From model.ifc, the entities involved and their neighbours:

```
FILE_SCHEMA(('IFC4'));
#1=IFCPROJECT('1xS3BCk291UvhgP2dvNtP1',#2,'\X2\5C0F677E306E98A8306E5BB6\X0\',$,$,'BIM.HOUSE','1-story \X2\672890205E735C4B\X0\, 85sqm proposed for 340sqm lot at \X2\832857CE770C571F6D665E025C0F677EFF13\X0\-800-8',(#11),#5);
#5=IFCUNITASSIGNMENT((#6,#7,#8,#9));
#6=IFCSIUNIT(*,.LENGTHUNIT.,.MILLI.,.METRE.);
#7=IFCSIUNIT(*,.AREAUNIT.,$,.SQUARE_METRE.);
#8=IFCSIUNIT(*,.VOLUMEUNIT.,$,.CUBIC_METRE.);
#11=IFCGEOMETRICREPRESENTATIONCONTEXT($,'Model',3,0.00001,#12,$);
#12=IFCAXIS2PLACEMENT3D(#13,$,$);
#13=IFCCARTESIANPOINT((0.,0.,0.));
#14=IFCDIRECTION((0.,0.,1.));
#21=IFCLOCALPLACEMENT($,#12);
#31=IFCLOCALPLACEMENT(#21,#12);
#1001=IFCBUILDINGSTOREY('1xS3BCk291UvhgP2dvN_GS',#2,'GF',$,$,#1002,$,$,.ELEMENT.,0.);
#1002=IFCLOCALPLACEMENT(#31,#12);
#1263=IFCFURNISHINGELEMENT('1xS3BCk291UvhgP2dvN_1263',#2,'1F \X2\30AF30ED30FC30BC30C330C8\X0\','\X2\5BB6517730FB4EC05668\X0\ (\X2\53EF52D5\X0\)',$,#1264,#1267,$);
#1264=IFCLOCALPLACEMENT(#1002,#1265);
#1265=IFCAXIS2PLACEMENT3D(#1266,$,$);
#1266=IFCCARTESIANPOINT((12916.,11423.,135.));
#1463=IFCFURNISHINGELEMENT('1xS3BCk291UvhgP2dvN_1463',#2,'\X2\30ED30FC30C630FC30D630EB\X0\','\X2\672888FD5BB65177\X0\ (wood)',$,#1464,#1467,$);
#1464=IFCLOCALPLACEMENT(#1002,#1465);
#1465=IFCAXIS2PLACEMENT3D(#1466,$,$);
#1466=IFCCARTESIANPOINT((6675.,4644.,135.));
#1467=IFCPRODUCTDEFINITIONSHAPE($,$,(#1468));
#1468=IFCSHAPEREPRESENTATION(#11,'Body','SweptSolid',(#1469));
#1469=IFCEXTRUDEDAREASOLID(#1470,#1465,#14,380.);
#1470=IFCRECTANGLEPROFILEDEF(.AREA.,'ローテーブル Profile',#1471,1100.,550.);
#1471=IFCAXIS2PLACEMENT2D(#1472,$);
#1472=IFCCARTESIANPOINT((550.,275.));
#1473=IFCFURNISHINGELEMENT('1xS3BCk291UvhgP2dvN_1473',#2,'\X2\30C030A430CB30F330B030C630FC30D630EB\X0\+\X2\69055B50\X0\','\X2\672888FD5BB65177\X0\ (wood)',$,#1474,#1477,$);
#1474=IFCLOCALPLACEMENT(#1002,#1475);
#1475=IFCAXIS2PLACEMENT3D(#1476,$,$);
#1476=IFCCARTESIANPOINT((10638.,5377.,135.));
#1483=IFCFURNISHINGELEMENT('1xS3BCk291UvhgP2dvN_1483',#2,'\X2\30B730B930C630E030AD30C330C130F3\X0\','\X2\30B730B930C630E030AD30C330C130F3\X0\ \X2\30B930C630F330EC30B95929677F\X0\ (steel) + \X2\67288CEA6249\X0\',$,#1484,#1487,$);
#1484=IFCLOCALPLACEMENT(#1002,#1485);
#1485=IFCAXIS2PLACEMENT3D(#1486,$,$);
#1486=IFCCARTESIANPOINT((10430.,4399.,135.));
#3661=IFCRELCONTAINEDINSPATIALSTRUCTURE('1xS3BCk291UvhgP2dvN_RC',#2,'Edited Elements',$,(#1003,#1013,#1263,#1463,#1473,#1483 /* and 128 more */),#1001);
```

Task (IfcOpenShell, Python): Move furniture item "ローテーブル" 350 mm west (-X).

```python
import ifcopenshell
import ifcopenshell.api.geometry
import ifcopenshell.util.placement

model = ifcopenshell.open("model.ifc")

item = model.by_id(1463)
matrix = ifcopenshell.util.placement.get_local_placement(item.ObjectPlacement)
matrix[0, 3] -= 350.0
ifcopenshell.api.geometry.edit_object_placement(model, product=item, matrix=matrix, is_si=False)

print(ifcopenshell.util.placement.get_local_placement(item.ObjectPlacement).round(3) + 0.0)

model.write("model_updated.ifc")
```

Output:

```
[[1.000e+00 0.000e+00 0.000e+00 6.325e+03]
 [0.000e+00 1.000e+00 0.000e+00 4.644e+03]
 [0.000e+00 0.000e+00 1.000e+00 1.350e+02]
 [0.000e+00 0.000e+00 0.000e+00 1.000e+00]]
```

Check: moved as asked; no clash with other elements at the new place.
